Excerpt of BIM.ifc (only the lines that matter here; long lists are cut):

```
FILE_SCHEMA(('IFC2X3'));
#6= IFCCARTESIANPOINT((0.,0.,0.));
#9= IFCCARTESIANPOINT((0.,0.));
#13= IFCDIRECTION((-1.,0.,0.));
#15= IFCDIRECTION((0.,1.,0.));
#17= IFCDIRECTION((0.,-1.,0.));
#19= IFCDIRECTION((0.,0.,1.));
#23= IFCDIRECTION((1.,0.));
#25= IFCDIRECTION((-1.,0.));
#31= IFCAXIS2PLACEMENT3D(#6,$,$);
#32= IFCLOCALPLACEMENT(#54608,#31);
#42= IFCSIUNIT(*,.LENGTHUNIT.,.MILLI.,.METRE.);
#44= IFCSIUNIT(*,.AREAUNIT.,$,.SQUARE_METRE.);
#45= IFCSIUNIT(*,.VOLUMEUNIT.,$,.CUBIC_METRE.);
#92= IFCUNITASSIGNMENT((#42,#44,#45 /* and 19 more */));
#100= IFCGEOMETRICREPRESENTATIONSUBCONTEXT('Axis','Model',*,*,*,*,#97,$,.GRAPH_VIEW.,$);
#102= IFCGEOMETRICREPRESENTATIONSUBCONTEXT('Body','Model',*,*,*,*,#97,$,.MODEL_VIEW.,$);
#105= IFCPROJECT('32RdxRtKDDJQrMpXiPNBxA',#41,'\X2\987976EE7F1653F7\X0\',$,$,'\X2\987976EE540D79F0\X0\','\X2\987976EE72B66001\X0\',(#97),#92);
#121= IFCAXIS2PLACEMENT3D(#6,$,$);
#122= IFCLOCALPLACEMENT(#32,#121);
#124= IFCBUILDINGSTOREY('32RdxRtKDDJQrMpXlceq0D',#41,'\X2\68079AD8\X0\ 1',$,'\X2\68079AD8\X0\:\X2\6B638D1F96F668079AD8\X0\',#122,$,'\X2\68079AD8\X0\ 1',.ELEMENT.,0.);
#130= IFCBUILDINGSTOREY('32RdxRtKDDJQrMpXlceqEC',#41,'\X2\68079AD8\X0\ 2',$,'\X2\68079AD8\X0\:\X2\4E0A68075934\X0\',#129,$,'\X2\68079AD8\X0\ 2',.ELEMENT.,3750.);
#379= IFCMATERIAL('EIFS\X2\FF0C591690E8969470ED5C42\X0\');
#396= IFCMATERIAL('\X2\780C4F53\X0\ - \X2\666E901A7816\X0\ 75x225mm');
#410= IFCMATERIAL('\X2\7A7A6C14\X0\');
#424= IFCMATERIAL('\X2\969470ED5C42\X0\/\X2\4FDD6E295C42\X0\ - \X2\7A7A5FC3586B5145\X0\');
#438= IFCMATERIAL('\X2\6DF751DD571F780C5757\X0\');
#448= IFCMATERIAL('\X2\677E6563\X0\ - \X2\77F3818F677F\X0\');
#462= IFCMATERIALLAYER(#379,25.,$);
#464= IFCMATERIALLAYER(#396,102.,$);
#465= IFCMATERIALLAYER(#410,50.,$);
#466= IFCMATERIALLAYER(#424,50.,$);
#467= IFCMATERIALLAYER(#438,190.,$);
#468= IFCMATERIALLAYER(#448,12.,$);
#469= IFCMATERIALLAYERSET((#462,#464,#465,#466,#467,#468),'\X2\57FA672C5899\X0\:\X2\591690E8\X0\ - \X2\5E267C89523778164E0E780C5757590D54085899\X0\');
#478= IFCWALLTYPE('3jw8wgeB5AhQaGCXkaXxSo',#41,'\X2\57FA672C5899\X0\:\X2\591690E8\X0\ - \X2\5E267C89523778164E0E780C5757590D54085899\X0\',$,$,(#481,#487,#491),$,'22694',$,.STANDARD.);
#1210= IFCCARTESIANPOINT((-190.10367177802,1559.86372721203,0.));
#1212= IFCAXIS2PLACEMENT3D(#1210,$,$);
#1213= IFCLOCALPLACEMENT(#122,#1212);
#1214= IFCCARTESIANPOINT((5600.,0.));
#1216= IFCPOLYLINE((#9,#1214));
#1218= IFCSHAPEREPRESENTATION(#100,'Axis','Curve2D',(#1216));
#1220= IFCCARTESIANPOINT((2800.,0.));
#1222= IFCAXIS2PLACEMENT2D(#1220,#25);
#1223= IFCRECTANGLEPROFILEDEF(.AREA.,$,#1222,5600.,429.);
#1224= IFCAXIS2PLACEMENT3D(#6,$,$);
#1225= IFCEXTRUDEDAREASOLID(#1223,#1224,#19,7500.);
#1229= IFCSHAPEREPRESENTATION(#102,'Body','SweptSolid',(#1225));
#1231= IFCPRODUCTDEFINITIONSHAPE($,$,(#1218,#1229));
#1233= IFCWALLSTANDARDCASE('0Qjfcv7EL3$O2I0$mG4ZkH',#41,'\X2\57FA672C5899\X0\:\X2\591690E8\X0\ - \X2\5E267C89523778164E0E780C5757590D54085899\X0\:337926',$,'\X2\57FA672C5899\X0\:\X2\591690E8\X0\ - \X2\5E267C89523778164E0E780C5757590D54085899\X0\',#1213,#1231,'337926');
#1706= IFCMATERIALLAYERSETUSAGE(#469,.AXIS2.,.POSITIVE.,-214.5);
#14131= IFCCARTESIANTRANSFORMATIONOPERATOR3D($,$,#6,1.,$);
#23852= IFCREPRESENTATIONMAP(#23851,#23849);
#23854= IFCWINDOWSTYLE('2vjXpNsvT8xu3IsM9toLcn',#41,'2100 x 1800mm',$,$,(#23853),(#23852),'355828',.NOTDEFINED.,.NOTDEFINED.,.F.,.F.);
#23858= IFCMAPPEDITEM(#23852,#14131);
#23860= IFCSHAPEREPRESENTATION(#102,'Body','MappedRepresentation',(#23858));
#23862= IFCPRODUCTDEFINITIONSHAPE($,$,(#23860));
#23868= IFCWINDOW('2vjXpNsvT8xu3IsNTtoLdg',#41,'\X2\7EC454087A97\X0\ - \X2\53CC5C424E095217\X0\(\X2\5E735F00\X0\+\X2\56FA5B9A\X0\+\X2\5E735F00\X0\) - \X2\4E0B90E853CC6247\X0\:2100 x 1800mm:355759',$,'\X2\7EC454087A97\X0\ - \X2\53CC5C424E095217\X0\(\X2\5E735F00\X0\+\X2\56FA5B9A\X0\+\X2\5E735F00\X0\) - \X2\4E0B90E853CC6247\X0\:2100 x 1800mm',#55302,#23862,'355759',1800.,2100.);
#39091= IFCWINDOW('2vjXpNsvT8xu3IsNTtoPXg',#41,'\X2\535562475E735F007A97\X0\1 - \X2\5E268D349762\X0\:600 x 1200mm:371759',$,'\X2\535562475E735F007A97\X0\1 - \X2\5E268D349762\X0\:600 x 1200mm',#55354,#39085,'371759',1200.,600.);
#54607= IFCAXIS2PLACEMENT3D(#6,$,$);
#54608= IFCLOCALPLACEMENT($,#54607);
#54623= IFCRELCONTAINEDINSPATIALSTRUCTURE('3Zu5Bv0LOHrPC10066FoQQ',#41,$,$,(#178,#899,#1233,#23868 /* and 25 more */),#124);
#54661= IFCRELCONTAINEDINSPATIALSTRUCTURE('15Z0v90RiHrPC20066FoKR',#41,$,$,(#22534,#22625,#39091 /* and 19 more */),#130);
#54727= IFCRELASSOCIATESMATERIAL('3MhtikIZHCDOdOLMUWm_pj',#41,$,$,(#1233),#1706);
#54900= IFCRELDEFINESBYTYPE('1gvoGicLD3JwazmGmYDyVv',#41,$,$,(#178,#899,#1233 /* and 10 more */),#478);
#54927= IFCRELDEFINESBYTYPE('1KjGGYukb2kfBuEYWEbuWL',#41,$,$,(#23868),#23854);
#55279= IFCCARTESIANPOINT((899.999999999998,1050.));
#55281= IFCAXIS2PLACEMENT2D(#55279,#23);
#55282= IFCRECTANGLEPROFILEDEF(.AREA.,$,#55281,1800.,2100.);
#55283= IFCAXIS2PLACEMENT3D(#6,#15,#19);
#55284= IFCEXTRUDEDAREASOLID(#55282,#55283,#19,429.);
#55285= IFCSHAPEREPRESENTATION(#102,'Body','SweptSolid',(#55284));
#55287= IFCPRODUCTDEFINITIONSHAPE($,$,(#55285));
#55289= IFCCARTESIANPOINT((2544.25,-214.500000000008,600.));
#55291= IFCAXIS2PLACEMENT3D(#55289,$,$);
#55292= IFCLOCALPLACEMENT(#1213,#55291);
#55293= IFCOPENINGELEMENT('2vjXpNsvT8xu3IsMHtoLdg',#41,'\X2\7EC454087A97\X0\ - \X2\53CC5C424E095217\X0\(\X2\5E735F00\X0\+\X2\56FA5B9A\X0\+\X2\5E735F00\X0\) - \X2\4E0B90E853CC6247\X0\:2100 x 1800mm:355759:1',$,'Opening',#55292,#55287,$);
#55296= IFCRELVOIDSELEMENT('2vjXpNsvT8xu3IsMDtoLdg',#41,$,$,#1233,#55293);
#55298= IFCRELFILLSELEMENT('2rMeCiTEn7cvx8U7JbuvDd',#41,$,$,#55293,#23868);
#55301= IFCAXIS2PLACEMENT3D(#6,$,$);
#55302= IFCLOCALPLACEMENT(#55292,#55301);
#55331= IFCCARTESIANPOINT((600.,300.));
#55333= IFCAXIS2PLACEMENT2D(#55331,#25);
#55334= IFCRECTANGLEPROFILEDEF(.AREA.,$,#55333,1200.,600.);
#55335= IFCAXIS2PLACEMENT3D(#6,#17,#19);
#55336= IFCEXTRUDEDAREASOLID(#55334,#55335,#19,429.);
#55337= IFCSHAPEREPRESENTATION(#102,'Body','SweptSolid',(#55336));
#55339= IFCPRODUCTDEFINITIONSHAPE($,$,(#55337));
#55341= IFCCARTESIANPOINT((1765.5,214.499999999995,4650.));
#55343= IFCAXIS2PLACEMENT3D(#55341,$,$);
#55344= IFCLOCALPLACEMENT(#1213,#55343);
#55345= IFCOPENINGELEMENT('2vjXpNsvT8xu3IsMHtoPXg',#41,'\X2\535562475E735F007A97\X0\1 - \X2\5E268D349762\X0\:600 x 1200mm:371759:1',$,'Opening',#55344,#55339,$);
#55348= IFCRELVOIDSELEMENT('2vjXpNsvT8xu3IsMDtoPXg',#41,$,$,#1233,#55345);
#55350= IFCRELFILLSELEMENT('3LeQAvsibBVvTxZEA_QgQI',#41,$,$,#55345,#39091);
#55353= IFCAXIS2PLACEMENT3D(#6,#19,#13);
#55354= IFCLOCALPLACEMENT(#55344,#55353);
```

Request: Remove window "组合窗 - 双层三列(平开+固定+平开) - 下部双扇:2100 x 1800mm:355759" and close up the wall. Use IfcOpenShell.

```python
import ifcopenshell
import ifcopenshell.api.feature
import ifcopenshell.api.root
import ifcopenshell.geom
import ifcopenshell.util.shape

model = ifcopenshell.open("BIM.ifc")
settings = ifcopenshell.geom.settings()


def volume(element):
    """Net volume in cubic metres, openings subtracted."""
    shape = ifcopenshell.geom.create_shape(settings, element)
    return ifcopenshell.util.shape.get_volume(shape.geometry)


window = model.by_id(23868)
opening = window.FillsVoids[0].RelatingOpeningElement
wall = opening.VoidsElements[0].RelatingBuildingElement
before = volume(wall)

ifcopenshell.api.root.remove_product(model, product=window)
ifcopenshell.api.feature.remove_feature(model, feature=opening)

after = volume(wall)

print(f"wall volume {before:.3f} -> {after:.3f} m3")

model.write("BIM_v2.ifc")
```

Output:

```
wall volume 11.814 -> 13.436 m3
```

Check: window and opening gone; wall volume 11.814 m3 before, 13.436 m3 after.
